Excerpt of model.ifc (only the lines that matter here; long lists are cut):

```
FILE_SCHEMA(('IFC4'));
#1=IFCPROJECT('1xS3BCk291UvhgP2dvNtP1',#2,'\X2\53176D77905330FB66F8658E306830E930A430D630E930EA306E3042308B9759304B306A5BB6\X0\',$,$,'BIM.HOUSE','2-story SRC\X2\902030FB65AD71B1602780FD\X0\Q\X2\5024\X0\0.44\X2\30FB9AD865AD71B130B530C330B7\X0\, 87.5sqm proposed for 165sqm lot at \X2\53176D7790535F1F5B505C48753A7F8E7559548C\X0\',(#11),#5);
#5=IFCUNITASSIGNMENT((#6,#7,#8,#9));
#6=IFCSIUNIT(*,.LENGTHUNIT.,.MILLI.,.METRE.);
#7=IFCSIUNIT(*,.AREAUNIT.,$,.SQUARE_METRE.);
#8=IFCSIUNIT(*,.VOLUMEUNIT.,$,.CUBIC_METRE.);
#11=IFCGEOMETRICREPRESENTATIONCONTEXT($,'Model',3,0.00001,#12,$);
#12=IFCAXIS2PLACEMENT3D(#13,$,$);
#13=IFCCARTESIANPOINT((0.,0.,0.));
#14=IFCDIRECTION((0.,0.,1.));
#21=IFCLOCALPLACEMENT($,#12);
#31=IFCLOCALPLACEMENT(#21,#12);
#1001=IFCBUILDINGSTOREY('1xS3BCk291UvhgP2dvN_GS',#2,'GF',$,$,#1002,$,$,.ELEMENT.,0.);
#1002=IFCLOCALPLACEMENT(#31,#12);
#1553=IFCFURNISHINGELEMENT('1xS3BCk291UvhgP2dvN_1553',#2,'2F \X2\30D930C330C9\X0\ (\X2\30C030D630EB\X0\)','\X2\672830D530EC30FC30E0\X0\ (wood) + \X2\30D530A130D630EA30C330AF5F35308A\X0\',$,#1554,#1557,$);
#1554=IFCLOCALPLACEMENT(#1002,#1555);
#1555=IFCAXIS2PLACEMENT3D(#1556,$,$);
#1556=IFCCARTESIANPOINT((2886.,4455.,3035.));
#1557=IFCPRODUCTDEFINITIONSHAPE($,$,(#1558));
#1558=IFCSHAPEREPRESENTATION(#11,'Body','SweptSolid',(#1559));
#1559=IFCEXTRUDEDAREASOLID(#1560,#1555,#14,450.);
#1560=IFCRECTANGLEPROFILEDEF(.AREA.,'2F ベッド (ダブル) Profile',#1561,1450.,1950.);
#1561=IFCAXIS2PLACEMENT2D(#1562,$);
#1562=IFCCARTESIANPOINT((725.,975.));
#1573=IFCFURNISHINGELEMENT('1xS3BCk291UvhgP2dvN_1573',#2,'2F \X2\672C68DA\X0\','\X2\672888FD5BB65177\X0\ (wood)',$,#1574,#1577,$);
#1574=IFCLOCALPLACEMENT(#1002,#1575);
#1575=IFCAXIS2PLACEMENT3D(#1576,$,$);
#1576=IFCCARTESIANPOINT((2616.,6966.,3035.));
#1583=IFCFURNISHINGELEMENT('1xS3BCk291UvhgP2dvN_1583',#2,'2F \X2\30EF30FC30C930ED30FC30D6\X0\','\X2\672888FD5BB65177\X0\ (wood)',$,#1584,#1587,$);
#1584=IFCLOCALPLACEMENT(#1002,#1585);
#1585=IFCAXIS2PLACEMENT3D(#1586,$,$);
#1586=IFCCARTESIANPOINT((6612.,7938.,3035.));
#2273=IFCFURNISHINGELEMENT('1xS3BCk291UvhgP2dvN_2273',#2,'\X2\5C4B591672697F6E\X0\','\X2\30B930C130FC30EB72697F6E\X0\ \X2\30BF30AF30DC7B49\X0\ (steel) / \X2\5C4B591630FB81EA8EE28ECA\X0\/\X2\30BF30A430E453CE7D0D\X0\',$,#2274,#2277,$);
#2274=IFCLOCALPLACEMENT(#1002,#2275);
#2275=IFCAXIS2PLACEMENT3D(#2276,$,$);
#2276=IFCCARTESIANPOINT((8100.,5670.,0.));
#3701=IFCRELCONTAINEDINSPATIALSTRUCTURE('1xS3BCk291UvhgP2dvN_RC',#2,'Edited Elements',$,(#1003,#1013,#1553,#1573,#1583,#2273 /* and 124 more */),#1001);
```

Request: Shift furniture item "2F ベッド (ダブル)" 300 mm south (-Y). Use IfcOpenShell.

```python
import ifcopenshell
import ifcopenshell.api.geometry
import ifcopenshell.util.placement

model = ifcopenshell.open("model.ifc")

item = model.by_guid("1xS3BCk291UvhgP2dvN_1553")
matrix = ifcopenshell.util.placement.get_local_placement(item.ObjectPlacement)
matrix[1, 3] -= 300.0
ifcopenshell.api.geometry.edit_object_placement(model, product=item, matrix=matrix, is_si=False)

print(ifcopenshell.util.placement.get_local_placement(item.ObjectPlacement).round(3) + 0.0)

model.write("model_updated.ifc")
```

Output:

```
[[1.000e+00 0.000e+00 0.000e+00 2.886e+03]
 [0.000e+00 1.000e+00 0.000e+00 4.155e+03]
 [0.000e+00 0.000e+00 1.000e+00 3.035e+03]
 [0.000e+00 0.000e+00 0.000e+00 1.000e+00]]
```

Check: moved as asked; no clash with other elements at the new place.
